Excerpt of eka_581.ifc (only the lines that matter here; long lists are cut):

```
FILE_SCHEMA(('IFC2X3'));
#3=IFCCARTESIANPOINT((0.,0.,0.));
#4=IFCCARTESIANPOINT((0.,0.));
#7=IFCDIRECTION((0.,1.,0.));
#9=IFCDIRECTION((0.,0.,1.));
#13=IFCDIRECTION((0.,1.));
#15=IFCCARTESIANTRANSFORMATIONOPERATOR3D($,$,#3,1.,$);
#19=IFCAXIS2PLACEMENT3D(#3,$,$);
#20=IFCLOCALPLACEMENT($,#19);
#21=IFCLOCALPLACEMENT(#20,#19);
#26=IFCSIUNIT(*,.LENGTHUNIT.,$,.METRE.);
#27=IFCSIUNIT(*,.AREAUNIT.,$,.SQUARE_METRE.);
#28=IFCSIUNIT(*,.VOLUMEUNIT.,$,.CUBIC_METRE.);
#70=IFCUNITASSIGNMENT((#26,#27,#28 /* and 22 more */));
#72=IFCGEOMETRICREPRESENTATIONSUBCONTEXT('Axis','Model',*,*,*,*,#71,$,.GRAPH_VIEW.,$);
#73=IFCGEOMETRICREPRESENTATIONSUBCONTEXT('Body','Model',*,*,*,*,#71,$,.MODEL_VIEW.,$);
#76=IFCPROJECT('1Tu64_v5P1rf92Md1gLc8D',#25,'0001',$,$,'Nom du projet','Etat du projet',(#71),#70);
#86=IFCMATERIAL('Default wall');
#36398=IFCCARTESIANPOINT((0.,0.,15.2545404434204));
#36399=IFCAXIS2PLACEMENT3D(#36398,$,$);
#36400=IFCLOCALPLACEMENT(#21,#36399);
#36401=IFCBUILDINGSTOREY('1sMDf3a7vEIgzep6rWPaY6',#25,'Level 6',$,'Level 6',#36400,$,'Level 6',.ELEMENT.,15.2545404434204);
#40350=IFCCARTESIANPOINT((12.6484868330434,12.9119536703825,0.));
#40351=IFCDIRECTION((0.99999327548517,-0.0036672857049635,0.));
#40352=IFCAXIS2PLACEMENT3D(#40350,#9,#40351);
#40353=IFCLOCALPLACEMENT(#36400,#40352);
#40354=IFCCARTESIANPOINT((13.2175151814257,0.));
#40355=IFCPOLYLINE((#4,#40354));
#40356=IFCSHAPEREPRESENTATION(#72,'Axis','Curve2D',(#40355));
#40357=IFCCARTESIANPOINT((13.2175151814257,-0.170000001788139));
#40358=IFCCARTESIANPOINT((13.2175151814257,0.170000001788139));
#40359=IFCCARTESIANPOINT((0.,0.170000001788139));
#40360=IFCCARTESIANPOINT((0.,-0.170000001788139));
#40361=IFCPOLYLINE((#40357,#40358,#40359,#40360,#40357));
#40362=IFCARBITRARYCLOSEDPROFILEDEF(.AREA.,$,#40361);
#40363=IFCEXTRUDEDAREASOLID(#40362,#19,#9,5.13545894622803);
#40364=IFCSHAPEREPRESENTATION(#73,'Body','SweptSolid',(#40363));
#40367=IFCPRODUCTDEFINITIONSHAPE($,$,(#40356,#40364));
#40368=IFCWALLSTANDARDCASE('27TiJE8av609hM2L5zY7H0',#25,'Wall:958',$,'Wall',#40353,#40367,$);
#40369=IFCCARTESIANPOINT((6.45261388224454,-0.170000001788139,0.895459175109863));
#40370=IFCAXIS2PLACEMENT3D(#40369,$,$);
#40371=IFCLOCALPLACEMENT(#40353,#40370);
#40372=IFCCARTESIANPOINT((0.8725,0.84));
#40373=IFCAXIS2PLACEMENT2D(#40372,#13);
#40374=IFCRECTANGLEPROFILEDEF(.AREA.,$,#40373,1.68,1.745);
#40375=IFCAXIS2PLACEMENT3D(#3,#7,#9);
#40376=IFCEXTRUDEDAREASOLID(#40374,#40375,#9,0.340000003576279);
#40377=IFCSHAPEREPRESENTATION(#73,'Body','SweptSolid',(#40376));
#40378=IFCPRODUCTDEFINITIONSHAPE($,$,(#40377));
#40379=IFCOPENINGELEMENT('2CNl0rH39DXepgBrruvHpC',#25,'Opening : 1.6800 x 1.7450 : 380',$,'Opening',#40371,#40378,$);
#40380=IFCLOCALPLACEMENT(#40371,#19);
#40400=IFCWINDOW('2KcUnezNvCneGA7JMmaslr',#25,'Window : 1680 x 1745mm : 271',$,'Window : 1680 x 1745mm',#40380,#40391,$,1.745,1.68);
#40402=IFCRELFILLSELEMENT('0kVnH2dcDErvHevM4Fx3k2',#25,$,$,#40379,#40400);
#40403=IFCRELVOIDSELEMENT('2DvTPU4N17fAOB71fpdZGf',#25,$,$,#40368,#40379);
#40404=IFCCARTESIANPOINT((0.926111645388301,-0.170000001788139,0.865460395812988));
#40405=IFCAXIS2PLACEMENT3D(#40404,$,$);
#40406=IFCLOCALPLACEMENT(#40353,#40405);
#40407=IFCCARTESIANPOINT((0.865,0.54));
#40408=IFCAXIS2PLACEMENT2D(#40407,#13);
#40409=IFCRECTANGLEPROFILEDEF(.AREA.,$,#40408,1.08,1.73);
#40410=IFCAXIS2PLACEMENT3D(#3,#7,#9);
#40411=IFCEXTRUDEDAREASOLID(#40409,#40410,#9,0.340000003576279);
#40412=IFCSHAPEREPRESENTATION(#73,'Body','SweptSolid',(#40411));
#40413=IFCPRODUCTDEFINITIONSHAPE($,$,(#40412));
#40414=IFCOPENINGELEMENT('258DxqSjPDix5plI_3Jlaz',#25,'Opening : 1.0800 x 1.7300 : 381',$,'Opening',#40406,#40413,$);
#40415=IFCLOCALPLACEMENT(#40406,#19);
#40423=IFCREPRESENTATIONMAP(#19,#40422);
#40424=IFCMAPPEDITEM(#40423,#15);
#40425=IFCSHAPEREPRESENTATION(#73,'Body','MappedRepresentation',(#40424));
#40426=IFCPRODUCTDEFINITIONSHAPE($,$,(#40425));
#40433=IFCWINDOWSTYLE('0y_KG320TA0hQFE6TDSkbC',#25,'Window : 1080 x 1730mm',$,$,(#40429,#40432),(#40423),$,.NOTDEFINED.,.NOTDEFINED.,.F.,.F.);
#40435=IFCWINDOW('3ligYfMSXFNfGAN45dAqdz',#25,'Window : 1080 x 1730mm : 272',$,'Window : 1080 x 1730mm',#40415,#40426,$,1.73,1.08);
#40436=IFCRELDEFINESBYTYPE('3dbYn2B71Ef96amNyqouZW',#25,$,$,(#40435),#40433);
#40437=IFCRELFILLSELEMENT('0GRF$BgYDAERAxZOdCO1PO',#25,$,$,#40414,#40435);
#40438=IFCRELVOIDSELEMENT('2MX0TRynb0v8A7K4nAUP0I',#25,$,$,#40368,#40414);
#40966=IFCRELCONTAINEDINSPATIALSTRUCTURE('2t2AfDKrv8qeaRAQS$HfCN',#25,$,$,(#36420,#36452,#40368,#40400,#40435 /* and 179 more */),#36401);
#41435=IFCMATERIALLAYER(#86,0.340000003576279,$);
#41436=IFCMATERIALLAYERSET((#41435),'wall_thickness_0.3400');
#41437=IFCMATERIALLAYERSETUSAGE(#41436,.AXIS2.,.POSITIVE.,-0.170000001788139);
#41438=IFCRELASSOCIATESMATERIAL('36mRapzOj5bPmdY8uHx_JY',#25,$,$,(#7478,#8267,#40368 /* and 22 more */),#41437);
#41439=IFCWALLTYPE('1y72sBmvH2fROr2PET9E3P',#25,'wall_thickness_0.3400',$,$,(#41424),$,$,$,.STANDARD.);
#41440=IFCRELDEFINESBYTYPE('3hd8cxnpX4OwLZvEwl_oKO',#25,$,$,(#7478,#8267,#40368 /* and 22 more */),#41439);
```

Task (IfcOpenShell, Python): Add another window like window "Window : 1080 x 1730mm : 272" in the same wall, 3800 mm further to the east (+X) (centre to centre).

```python
import ifcopenshell
import ifcopenshell.api.feature
import ifcopenshell.api.geometry
import ifcopenshell.api.root
import ifcopenshell.geom
import ifcopenshell.util.element
import ifcopenshell.util.placement
import ifcopenshell.util.shape

model = ifcopenshell.open("eka_581.ifc")
settings = ifcopenshell.geom.settings()


def volume(element):
    """Net volume in cubic metres, openings subtracted."""
    shape = ifcopenshell.geom.create_shape(settings, element)
    return ifcopenshell.util.shape.get_volume(shape.geometry)


window = model.by_guid("3ligYfMSXFNfGAN45dAqdz")
opening = window.FillsVoids[0].RelatingOpeningElement
wall = opening.VoidsElements[0].RelatingBuildingElement
before = volume(wall)
shift = ifcopenshell.util.placement.get_local_placement(wall.ObjectPlacement)[:3, 0] * 3.8

# copy_class copies the void relationship, type, container and properties, but no geometry.
new_opening = ifcopenshell.api.root.copy_class(model, product=opening)
new_opening.Representation = ifcopenshell.util.element.copy_deep(
    model, opening.Representation, exclude=["IfcGeometricRepresentationContext", "IfcRepresentationMap"]
)
new_opening.Name = "Opening : 1.0800 x 1.7300"
new_window = ifcopenshell.api.root.copy_class(model, product=window)
new_window.Representation = ifcopenshell.util.element.copy_deep(
    model, window.Representation, exclude=["IfcGeometricRepresentationContext", "IfcRepresentationMap"]
)
new_window.Name = "Window : 1080 x 1730mm"
fills = ifcopenshell.api.feature.add_filling(model, opening=new_opening, element=new_window)
fills.OwnerHistory = new_window.OwnerHistory  # required in IFC2X3

for old, new in ((opening, new_opening), (window, new_window)):
    matrix = ifcopenshell.util.placement.get_local_placement(old.ObjectPlacement)
    matrix[:3, 3] += shift
    ifcopenshell.api.geometry.edit_object_placement(model, product=new, matrix=matrix, is_si=False)

after = volume(wall)

print(f"wall volume {before:.3f} -> {after:.3f} m3")

model.write("eka_581_rev.ifc")
```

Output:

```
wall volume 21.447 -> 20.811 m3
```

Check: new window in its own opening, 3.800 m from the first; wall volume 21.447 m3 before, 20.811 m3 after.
